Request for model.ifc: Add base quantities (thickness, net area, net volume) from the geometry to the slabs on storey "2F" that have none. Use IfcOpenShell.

First a look at what the model holds.

```python
import ifcopenshell
import ifcopenshell.util.element
import ifcopenshell.util.unit

model = ifcopenshell.open("model.ifc")
print(model.schema)
for unit_type in ("LENGTHUNIT", "AREAUNIT", "VOLUMEUNIT"):
    print(unit_type, ifcopenshell.util.unit.calculate_unit_scale(model, unit_type))
storey = next(s for s in model.by_type("IfcBuildingStorey") if s.Name == "2F")
slabs = [e for e in ifcopenshell.util.element.get_decomposition(storey) if e.is_a("IfcSlab")]
for e in sorted(slabs, key=lambda e: e.id()):
    print(e.id(), e.is_a(), e.Name, list(ifcopenshell.util.element.get_psets(e, qtos_only=True)), sep=" | ")
```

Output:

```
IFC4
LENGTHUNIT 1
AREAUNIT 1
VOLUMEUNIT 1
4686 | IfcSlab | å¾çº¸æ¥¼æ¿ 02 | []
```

```python
import ifcopenshell
import ifcopenshell.api.pset
import ifcopenshell.geom
import ifcopenshell.util.element
import ifcopenshell.util.shape
import ifcopenshell.util.unit

model = ifcopenshell.open("model.ifc")
unit_scale = ifcopenshell.util.unit.calculate_unit_scale(model)
area_scale = ifcopenshell.util.unit.calculate_unit_scale(model, "AREAUNIT")
volume_scale = ifcopenshell.util.unit.calculate_unit_scale(model, "VOLUMEUNIT")
settings = ifcopenshell.geom.settings()

storey = next(s for s in model.by_type("IfcBuildingStorey") if s.Name == "2F")
slabs = [e for e in ifcopenshell.util.element.get_decomposition(storey) if e.is_a("IfcSlab")]

for e in sorted(slabs, key=lambda e: e.id()):
    if ifcopenshell.util.element.get_psets(e, qtos_only=True, should_inherit=False):
        continue
    # Geometry comes back in metres, in the element's own axes.
    shape = ifcopenshell.geom.create_shape(settings, e)
    values = {
        "Width": ifcopenshell.util.shape.get_z(shape.geometry) / unit_scale,
        "NetArea": ifcopenshell.util.shape.get_footprint_area(shape.geometry) / area_scale,
        "NetVolume": ifcopenshell.util.shape.get_volume(shape.geometry) / volume_scale,
    }
    qto = ifcopenshell.api.pset.add_qto(model, product=e, name="Qto_SlabBaseQuantities")
    ifcopenshell.api.pset.edit_qto(model, qto=qto, properties=values)
    print(e.id(), {k: round(v, 3) for k, v in values.items()})

model.write("model-out.ifc")
```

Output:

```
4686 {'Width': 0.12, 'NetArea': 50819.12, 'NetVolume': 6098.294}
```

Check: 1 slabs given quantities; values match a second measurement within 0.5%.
